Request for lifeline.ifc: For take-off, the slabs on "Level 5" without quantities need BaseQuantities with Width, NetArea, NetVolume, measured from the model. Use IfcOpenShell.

First a look at what the model holds.

```python
import ifcopenshell
import ifcopenshell.util.element
import ifcopenshell.util.unit

model = ifcopenshell.open("lifeline.ifc")
print(model.schema)
for unit_type in ("LENGTHUNIT", "AREAUNIT", "VOLUMEUNIT"):
    print(unit_type, ifcopenshell.util.unit.calculate_unit_scale(model, unit_type))
storey = next(s for s in model.by_type("IfcBuildingStorey") if s.Name == "Level 5")
slabs = [e for e in ifcopenshell.util.element.get_decomposition(storey) if e.is_a("IfcSlab")]
for e in sorted(slabs, key=lambda e: e.id()):
    print(e.id(), e.is_a(), e.Name, list(ifcopenshell.util.element.get_psets(e, qtos_only=True)), sep=" | ")
```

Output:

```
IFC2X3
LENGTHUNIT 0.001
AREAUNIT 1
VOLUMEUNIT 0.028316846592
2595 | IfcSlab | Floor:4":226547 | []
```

```python
import ifcopenshell
import ifcopenshell.api.pset
import ifcopenshell.geom
import ifcopenshell.util.element
import ifcopenshell.util.shape
import ifcopenshell.util.unit

model = ifcopenshell.open("lifeline.ifc")
unit_scale = ifcopenshell.util.unit.calculate_unit_scale(model)
area_scale = ifcopenshell.util.unit.calculate_unit_scale(model, "AREAUNIT")
volume_scale = ifcopenshell.util.unit.calculate_unit_scale(model, "VOLUMEUNIT")
settings = ifcopenshell.geom.settings()

storey = next(s for s in model.by_type("IfcBuildingStorey") if s.Name == "Level 5")
slabs = [e for e in ifcopenshell.util.element.get_decomposition(storey) if e.is_a("IfcSlab")]

for e in sorted(slabs, key=lambda e: e.id()):
    if ifcopenshell.util.element.get_psets(e, qtos_only=True, should_inherit=False):
        continue
    # Geometry comes back in metres, in the element's own axes.
    shape = ifcopenshell.geom.create_shape(settings, e)
    values = {
        "Width": ifcopenshell.util.shape.get_z(shape.geometry) / unit_scale,
        "NetArea": ifcopenshell.util.shape.get_footprint_area(shape.geometry) / area_scale,
        "NetVolume": ifcopenshell.util.shape.get_volume(shape.geometry) / volume_scale,
    }
    qto = ifcopenshell.api.pset.add_qto(model, product=e, name="BaseQuantities")
    ifcopenshell.api.pset.edit_qto(model, qto=qto, properties=values)
    print(e.id(), {k: round(v, 3) for k, v in values.items()})

model.write("lifeline_v2.ifc")
```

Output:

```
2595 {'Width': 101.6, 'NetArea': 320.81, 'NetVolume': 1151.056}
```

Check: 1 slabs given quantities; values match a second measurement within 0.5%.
